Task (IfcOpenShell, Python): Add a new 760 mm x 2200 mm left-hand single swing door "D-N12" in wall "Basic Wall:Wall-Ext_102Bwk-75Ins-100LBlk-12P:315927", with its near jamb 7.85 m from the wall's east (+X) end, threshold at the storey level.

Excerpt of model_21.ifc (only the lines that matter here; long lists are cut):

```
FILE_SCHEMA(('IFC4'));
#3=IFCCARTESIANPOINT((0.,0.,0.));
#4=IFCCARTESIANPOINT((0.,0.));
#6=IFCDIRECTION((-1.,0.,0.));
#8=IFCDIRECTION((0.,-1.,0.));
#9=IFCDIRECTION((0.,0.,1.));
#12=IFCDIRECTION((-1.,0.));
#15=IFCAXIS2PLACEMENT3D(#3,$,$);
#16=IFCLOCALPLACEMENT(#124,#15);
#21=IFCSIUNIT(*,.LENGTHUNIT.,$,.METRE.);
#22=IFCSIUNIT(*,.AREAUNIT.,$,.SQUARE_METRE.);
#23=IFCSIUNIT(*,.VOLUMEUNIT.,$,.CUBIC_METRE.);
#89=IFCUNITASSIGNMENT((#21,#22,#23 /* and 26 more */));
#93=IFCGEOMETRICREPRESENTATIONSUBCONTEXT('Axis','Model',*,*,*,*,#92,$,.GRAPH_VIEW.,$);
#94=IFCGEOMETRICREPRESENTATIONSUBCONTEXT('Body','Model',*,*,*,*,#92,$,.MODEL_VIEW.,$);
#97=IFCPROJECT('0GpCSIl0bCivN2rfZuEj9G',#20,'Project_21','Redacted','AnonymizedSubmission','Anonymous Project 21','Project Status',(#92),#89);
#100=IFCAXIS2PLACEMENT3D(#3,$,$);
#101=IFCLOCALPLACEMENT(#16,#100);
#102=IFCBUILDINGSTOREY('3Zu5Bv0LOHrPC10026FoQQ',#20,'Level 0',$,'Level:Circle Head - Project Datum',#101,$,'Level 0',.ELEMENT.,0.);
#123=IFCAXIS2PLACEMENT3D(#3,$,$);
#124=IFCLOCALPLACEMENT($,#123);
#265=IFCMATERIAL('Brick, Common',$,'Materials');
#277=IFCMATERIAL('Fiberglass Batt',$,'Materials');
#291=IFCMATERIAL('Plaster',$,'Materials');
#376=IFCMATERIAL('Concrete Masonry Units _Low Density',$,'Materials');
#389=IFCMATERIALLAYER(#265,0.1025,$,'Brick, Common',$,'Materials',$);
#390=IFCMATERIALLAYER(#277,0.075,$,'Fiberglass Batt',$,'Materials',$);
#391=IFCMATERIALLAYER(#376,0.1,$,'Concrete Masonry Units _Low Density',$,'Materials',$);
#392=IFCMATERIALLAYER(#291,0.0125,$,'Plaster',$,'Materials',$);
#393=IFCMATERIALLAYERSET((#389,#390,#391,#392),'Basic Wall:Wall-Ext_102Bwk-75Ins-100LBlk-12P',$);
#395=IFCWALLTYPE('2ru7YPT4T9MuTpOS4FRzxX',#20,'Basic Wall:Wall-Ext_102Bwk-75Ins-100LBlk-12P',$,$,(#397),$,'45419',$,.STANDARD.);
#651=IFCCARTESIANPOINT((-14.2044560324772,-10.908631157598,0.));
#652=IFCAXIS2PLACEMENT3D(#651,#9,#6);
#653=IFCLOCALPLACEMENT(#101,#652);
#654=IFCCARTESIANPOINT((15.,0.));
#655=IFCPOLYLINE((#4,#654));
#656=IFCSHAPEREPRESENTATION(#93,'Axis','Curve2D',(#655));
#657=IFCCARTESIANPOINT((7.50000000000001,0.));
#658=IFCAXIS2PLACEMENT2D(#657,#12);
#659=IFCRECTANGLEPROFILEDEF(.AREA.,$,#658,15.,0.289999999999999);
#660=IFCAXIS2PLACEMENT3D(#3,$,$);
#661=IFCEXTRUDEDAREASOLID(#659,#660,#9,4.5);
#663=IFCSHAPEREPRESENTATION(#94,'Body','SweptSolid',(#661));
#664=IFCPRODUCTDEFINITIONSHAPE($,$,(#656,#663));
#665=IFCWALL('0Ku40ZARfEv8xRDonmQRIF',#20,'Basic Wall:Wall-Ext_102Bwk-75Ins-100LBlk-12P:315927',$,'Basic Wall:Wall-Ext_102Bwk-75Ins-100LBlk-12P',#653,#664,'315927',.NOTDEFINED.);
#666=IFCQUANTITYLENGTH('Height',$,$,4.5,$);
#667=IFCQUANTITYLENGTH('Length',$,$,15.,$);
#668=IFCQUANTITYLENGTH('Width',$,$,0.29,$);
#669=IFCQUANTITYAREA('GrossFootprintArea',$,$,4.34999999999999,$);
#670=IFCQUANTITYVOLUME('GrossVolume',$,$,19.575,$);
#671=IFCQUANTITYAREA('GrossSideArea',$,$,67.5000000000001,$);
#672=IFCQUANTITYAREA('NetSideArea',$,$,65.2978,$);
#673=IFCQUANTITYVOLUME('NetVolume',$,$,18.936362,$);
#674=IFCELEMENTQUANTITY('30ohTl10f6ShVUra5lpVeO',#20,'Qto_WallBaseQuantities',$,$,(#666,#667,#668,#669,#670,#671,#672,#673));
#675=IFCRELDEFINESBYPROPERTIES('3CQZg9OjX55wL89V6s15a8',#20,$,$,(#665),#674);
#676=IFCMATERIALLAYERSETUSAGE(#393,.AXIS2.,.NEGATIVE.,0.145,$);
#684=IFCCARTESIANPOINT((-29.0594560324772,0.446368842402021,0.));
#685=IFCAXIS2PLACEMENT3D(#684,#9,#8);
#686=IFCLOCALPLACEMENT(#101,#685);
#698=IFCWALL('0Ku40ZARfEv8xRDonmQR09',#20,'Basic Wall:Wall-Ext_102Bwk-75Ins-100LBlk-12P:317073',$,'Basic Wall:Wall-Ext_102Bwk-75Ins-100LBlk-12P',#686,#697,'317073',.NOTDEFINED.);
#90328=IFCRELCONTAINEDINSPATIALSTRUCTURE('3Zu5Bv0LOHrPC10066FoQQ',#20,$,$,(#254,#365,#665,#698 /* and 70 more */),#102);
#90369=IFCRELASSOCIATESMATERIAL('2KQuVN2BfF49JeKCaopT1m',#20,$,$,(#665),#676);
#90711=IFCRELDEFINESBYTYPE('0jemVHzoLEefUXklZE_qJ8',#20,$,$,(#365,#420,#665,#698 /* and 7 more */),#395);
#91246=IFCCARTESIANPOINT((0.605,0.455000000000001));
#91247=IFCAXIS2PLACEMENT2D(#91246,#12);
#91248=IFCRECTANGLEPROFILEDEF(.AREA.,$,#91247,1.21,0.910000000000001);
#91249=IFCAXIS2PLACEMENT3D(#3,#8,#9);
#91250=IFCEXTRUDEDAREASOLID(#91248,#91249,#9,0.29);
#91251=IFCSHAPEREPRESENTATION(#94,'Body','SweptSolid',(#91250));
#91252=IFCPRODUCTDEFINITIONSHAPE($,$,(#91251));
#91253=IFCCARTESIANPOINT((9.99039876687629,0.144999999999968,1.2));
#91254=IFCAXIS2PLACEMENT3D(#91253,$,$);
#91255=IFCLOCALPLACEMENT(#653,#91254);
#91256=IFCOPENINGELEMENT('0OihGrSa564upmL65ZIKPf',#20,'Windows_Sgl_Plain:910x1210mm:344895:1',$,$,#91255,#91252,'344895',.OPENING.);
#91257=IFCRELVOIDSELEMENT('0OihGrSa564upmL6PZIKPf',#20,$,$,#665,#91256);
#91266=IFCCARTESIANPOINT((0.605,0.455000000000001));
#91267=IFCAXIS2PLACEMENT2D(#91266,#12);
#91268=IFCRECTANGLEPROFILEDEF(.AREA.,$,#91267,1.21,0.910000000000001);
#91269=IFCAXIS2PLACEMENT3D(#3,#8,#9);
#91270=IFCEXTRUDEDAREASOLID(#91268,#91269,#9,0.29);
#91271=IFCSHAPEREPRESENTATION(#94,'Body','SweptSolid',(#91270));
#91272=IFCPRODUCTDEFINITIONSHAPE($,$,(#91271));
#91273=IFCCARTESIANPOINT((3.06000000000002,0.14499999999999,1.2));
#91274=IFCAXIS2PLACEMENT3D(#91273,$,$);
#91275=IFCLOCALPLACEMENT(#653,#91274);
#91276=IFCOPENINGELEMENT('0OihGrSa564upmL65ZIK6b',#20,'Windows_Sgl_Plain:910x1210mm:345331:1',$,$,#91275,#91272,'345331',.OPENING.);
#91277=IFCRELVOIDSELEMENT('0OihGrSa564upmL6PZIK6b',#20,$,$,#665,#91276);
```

```python
import numpy as np
import ifcopenshell
import ifcopenshell.api.feature
import ifcopenshell.api.geometry
import ifcopenshell.api.pset
import ifcopenshell.api.root
import ifcopenshell.api.spatial
import ifcopenshell.geom
import ifcopenshell.util.element
import ifcopenshell.util.placement
import ifcopenshell.util.representation
import ifcopenshell.util.shape
import ifcopenshell.util.unit

model = ifcopenshell.open("model_21.ifc")
unit_scale = ifcopenshell.util.unit.calculate_unit_scale(model)
area_scale = ifcopenshell.util.unit.calculate_unit_scale(model, "AREAUNIT")
volume_scale = ifcopenshell.util.unit.calculate_unit_scale(model, "VOLUMEUNIT")
settings = ifcopenshell.geom.settings()


def volume(element):
    """Net volume in cubic metres, openings subtracted."""
    shape = ifcopenshell.geom.create_shape(settings, element)
    return ifcopenshell.util.shape.get_volume(shape.geometry)


wall = model.by_guid("0Ku40ZARfEv8xRDonmQRIF")
storey = ifcopenshell.util.element.get_container(wall, ifc_class="IfcBuildingStorey")
context = ifcopenshell.util.representation.get_context(model, "Model", "Body", "MODEL_VIEW")
before = volume(wall)

width, height, from_end, sill = 0.76, 2.2, 7.85, 0.0  # metres

# The wall runs along its own X axis, and the end named is its -X end.
wall_shape = ifcopenshell.geom.create_shape(settings, wall)
x, y, z = ifcopenshell.util.shape.get_vertices(wall_shape.geometry).T
start = x.min() + from_end
face, thickness = float(y.min()), float(y.max() - y.min())
wall_matrix = ifcopenshell.util.placement.get_local_placement(wall.ObjectPlacement)
level = ifcopenshell.util.placement.get_local_placement(storey.ObjectPlacement)[2, 3]


def in_wall(x, y):
    """Placement at x, y metres in the wall's axes, at sill height."""
    matrix = wall_matrix.copy()
    matrix[:, 3] = wall_matrix @ np.array([x / unit_scale, y / unit_scale, 0.0, 1.0])
    matrix[2, 3] = level + sill / unit_scale
    return matrix


# Opening: a box that overshoots both wall faces by 50 mm.
opening = ifcopenshell.api.root.create_entity(model, ifc_class="IfcOpeningElement", predefined_type="OPENING")
box = ifcopenshell.api.geometry.add_wall_representation(
    model, context=context, length=width, height=height, thickness=thickness + 0.1
)
ifcopenshell.api.geometry.assign_representation(model, product=opening, representation=box)
ifcopenshell.api.geometry.edit_object_placement(model, product=opening, matrix=in_wall(start, face - 0.05), is_si=False)
ifcopenshell.api.feature.add_feature(model, feature=opening, element=wall)

door = ifcopenshell.api.root.create_entity(model, ifc_class="IfcDoor", name="D-N12", predefined_type="DOOR")
door.OverallWidth, door.OverallHeight = width / unit_scale, height / unit_scale
door.OperationType = "SINGLE_SWING_LEFT"
body = ifcopenshell.api.geometry.add_door_representation(
    model,
    context=context,
    overall_width=door.OverallWidth,
    overall_height=door.OverallHeight,
    operation_type="SINGLE_SWING_LEFT",
    lining_properties={"LiningDepth": thickness / unit_scale, "ThresholdDepth": thickness / unit_scale},
)
ifcopenshell.api.geometry.assign_representation(model, product=door, representation=body)
ifcopenshell.api.spatial.assign_container(model, products=[door], relating_structure=storey)
ifcopenshell.api.feature.add_filling(model, opening=opening, element=door)

# The lining spans the wall, so the door starts at the wall face.
ifcopenshell.api.geometry.edit_object_placement(model, product=door, matrix=in_wall(start, face), is_si=False)

after = volume(wall)

# Update the wall's stored quantities.
qto = model.by_id(ifcopenshell.util.element.get_pset(wall, "Qto_WallBaseQuantities", should_inherit=False)["id"])
ifcopenshell.api.pset.edit_qto(model, qto=qto, properties={
    "NetSideArea": after / thickness / area_scale,
    "NetVolume": after / volume_scale,
})

print(f"wall volume {before:.3f} -> {after:.3f} m3")

model.write("model_21_updated.ifc")
```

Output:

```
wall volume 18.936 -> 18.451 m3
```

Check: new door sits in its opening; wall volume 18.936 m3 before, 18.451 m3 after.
